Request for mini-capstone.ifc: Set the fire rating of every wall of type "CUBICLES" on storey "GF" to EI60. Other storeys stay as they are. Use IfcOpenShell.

First a look at what the model holds.

```python
import ifcopenshell
import ifcopenshell.util.element

model = ifcopenshell.open("mini-capstone.ifc")
print(model.schema)
storey = next(s for s in model.by_type("IfcBuildingStorey") if s.Name == "GF")
walls = [e for e in ifcopenshell.util.element.get_decomposition(storey) if e.is_a("IfcWall")]
seen = {}
for e in walls:
    element_type = ifcopenshell.util.element.get_type(e)
    key = (element_type.Name if element_type != e and element_type else None, ifcopenshell.util.element.get_pset(e, "Pset_WallCommon", "FireRating"))
    seen[key] = seen.get(key, 0) + 1
for (name, value), count in sorted(seen.items(), key=str):
    print(count, "x", name, "|", value)
```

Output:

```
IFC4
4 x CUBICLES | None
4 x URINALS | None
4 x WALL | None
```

```python
import ifcopenshell
import ifcopenshell.api.pset
import ifcopenshell.util.element

model = ifcopenshell.open("mini-capstone.ifc")

storey = next(s for s in model.by_type("IfcBuildingStorey") if s.Name == "GF")
walls = [e for e in ifcopenshell.util.element.get_decomposition(storey) if e.is_a("IfcWall")]

count = 0
for e in walls:
    element_type = ifcopenshell.util.element.get_type(e)
    if element_type in (None, e) or element_type.Name != "CUBICLES":
        continue
    # add_pset returns the element's existing set when there is one.
    pset = ifcopenshell.api.pset.add_pset(model, product=e, name="Pset_WallCommon")
    ifcopenshell.api.pset.edit_pset(model, pset=pset, properties={"FireRating": "EI60"})
    count += 1

print(count, "walls updated")

model.write("mini-capstone-out.ifc")
```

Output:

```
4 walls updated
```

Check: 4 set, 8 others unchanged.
